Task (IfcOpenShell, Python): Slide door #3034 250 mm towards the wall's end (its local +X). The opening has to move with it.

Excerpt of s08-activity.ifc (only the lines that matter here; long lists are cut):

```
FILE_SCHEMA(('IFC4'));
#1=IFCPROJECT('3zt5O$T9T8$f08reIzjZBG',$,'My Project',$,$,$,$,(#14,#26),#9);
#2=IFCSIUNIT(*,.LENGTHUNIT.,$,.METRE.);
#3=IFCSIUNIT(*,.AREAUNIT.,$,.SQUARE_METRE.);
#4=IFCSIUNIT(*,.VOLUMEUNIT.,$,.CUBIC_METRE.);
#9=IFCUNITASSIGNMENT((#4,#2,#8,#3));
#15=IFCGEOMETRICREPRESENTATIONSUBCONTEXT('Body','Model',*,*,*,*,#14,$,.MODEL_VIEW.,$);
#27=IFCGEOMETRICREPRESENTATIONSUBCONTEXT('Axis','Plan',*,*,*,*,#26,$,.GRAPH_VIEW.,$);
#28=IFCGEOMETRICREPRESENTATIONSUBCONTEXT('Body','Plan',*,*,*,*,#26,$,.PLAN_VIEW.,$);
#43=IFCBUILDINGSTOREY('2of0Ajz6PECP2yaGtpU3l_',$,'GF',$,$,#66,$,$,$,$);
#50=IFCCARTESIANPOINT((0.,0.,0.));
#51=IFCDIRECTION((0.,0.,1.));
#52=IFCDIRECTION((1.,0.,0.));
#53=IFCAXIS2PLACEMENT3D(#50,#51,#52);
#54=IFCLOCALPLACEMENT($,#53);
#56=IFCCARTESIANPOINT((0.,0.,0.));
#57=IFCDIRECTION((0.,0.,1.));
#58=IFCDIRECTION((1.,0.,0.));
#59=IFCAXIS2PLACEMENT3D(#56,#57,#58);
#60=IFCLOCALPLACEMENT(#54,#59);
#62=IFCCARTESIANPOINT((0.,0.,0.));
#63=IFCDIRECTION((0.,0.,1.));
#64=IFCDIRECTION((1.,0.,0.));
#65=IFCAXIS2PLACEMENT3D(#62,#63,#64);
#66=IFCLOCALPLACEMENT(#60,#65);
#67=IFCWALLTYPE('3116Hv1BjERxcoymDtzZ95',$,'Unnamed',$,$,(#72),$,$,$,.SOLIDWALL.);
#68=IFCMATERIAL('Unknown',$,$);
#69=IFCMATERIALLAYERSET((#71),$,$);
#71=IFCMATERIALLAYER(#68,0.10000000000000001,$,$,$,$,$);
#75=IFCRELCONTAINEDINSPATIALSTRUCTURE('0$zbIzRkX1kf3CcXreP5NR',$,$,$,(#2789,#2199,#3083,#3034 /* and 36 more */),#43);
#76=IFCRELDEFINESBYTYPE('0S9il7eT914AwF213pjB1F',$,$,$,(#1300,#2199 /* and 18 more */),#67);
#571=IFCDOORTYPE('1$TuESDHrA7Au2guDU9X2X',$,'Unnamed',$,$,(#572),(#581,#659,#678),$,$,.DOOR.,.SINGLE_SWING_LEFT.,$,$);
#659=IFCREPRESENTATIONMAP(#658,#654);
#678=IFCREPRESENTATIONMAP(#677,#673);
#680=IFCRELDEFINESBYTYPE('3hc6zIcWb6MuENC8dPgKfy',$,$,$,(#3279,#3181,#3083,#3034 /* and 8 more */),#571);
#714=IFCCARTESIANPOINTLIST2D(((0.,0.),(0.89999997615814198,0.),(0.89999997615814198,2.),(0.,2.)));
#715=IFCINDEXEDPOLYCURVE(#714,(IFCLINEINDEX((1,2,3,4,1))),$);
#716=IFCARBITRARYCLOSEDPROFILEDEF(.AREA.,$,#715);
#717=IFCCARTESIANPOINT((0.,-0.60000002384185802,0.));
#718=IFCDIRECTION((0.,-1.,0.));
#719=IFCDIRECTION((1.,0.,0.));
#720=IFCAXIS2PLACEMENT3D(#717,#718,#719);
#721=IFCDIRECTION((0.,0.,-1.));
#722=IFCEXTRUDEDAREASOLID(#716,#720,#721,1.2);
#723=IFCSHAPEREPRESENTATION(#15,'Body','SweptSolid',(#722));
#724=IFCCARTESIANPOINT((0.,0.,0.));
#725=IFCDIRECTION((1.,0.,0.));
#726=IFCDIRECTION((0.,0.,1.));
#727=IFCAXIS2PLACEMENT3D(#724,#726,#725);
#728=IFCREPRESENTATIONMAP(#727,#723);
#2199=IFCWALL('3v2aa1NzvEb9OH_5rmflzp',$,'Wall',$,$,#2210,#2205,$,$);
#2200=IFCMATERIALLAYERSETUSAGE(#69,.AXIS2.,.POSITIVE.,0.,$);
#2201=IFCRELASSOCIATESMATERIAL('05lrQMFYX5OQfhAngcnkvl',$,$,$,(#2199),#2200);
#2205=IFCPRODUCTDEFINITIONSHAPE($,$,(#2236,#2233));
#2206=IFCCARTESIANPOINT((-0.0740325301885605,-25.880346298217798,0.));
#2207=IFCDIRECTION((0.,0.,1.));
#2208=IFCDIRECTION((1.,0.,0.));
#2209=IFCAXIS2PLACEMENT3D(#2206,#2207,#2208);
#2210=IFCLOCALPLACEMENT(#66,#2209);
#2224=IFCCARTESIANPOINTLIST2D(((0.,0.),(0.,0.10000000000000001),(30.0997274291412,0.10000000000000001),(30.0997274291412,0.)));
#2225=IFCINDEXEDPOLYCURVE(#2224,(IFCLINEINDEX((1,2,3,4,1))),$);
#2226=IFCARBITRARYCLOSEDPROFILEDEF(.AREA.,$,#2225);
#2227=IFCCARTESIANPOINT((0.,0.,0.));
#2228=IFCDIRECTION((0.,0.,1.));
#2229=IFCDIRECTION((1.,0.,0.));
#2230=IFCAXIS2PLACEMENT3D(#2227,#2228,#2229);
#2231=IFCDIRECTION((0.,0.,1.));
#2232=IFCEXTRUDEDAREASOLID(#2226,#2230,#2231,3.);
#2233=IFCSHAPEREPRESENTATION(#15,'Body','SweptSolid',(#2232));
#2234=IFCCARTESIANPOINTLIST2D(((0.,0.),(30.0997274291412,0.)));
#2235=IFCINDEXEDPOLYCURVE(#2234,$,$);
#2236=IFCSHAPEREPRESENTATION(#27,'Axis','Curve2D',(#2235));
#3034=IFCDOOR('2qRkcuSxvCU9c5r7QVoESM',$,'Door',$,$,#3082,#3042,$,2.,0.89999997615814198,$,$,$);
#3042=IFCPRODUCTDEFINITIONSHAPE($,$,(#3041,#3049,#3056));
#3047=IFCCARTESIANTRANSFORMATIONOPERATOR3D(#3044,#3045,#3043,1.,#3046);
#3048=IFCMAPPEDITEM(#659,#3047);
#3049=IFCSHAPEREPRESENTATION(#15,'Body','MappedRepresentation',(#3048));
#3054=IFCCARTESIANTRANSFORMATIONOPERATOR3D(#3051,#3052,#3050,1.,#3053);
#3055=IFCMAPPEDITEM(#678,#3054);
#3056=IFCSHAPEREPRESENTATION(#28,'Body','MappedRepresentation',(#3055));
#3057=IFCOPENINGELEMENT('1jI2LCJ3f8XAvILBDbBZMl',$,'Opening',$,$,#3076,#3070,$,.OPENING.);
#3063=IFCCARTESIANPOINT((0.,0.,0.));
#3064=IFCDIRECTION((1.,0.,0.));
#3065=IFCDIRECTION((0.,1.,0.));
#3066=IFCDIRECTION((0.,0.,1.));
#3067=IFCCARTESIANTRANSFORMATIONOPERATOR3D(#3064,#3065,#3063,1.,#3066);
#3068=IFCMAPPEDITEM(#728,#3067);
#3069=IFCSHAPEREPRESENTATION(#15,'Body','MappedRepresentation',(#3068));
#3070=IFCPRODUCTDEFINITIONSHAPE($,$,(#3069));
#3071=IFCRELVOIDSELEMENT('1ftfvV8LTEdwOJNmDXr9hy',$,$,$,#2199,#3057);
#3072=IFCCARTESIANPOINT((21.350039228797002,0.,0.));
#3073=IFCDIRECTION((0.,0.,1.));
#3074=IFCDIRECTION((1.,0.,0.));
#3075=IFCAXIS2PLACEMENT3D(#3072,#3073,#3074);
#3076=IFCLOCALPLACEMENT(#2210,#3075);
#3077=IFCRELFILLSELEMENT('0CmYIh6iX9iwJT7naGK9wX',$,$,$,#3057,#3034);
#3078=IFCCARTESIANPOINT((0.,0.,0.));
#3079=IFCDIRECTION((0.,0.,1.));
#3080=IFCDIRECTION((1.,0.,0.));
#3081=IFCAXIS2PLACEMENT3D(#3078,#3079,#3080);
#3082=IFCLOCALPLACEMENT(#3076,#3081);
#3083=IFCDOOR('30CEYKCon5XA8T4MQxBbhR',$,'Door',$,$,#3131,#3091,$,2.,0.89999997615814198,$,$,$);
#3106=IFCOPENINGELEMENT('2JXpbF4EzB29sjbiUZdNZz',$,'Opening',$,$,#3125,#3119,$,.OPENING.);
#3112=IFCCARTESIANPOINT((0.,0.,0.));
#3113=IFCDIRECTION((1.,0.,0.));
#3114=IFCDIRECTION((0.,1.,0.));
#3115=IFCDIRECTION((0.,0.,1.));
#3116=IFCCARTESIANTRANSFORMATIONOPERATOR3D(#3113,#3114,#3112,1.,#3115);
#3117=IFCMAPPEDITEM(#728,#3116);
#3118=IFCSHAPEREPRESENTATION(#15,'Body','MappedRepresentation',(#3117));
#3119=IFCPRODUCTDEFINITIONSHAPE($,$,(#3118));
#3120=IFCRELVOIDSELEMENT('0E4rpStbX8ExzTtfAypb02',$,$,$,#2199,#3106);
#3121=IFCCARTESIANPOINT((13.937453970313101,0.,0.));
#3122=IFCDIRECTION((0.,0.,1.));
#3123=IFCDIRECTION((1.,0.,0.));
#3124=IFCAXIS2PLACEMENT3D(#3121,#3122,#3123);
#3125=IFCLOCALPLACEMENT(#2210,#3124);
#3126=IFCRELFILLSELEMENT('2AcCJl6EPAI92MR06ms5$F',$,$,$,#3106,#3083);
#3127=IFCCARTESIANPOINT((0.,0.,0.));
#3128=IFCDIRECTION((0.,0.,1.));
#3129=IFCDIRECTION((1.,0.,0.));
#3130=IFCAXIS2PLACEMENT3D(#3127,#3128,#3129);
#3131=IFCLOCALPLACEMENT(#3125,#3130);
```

```python
import ifcopenshell
import ifcopenshell.api.geometry
import ifcopenshell.util.placement
import ifcopenshell.util.unit

model = ifcopenshell.open("s08-activity.ifc")
unit_scale = ifcopenshell.util.unit.calculate_unit_scale(model)

door = model.by_guid("2qRkcuSxvCU9c5r7QVoESM")
opening = door.FillsVoids[0].RelatingOpeningElement
wall = opening.VoidsElements[0].RelatingBuildingElement

wall_matrix = ifcopenshell.util.placement.get_local_placement(wall.ObjectPlacement)
shift = wall_matrix[:3, 0] * 0.25 / unit_scale
before = ifcopenshell.util.placement.get_local_placement(door.ObjectPlacement)[:3, 3].copy()

# The door is placed relative to its opening, so it follows when the opening moves.
matrix = ifcopenshell.util.placement.get_local_placement(opening.ObjectPlacement)
matrix[:3, 3] += shift
ifcopenshell.api.geometry.edit_object_placement(
    model, product=opening, matrix=matrix, is_si=False, should_transform_children=True
)

after = ifcopenshell.util.placement.get_local_placement(door.ObjectPlacement)[:3, 3]
print("door moved by", (after - before).round(3) + 0.0)

model.write("s08-activity_updated.ifc")
```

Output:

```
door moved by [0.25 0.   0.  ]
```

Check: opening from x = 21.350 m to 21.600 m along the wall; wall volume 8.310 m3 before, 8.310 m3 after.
